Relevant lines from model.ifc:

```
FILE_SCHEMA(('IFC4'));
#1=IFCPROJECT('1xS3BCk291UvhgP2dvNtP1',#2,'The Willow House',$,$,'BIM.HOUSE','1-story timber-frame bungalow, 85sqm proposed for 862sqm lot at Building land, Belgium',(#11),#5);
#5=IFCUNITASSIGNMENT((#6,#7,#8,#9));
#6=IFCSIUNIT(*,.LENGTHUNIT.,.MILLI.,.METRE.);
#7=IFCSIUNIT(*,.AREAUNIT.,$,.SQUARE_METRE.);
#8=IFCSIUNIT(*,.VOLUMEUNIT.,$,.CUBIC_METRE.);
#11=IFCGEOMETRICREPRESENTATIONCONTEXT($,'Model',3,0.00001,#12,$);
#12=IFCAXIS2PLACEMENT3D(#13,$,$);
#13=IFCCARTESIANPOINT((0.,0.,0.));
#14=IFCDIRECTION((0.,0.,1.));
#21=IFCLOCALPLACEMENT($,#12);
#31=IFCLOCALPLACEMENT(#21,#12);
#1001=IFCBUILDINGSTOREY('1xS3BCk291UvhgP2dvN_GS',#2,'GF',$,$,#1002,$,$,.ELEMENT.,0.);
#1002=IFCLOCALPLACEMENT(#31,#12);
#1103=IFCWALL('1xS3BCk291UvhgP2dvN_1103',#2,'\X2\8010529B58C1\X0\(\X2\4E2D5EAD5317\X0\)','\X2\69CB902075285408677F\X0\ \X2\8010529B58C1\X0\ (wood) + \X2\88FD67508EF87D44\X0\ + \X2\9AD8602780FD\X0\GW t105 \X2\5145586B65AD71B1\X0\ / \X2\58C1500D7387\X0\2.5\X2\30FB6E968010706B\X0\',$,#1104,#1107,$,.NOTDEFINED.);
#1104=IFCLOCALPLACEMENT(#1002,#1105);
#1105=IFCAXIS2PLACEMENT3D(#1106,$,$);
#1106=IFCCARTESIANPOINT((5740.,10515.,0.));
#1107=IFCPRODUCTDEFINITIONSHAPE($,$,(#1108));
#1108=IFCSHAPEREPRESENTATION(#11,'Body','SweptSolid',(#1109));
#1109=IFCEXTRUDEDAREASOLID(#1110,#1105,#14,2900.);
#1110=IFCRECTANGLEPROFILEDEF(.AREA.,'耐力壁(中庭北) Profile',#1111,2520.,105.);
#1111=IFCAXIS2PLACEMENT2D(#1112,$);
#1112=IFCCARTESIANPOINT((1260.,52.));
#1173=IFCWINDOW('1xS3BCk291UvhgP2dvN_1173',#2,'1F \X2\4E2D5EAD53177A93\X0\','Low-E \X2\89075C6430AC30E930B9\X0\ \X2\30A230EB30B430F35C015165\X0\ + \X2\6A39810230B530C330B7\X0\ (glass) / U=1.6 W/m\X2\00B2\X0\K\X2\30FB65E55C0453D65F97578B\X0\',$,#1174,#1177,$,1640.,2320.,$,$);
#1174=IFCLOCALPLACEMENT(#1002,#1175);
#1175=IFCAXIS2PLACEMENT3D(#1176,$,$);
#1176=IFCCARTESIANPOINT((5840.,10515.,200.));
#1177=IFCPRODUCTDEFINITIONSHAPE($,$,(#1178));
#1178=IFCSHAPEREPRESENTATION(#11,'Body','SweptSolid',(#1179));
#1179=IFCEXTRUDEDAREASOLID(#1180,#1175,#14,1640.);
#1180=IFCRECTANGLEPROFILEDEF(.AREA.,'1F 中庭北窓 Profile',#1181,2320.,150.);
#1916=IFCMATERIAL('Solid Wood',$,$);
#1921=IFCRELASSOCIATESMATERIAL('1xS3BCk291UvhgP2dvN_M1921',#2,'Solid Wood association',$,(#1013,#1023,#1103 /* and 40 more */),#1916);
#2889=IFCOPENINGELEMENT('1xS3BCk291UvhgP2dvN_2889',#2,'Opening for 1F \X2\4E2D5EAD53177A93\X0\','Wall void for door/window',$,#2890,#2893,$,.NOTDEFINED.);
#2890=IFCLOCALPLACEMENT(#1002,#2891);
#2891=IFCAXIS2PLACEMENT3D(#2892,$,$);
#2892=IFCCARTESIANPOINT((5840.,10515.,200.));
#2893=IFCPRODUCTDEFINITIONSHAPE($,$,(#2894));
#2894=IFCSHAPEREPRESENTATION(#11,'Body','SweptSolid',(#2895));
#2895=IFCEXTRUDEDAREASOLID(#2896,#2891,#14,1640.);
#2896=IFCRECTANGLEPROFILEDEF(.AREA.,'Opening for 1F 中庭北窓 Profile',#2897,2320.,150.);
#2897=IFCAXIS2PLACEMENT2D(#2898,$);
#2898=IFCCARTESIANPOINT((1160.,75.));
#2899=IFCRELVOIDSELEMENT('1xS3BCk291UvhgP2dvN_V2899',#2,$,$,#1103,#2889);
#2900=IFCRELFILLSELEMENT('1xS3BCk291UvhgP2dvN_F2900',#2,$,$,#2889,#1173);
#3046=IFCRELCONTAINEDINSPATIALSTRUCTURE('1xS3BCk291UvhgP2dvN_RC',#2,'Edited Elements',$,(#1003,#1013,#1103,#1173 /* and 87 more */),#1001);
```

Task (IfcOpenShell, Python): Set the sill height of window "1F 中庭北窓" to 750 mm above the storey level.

```python
import numpy as np
import ifcopenshell
import ifcopenshell.api.geometry
import ifcopenshell.geom
import ifcopenshell.util.element
import ifcopenshell.util.placement
import ifcopenshell.util.shape
import ifcopenshell.util.unit

model = ifcopenshell.open("model.ifc")
unit_scale = ifcopenshell.util.unit.calculate_unit_scale(model)

window = model.by_guid("1xS3BCk291UvhgP2dvN_1173")
opening = window.FillsVoids[0].RelatingOpeningElement
storey = ifcopenshell.util.element.get_container(window, ifc_class="IfcBuildingStorey")
level = ifcopenshell.util.placement.get_local_placement(storey.ObjectPlacement)[2, 3]

# The opening's origin need not be at the sill, so measure its lowest point.
shape = ifcopenshell.geom.create_shape(ifcopenshell.geom.settings(), opening)
bottom = ifcopenshell.util.shape.get_shape_bottom_elevation(shape, shape.geometry) / unit_scale
dz = level + 0.75 / unit_scale - bottom

shift = np.array([0.0, 0.0, dz])
# The window is not placed relative to its opening, so move both.
for product in (opening, window):
    matrix = ifcopenshell.util.placement.get_local_placement(product.ObjectPlacement)
    matrix[:3, 3] += shift
    ifcopenshell.api.geometry.edit_object_placement(model, product=product, matrix=matrix, is_si=False)

print(f"moved by {dz * unit_scale:+.3f} m")

model.write("model_edited.ifc")
```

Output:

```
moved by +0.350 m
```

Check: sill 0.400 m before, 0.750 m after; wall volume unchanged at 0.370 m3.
